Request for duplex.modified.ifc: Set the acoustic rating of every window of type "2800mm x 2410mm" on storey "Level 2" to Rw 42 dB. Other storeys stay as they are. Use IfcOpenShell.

First a look at what the model holds.

```python
import ifcopenshell
import ifcopenshell.util.element

model = ifcopenshell.open("duplex.modified.ifc")
print(model.schema)
storey = next(s for s in model.by_type("IfcBuildingStorey") if s.Name == "Level 2")
windows = [e for e in ifcopenshell.util.element.get_decomposition(storey) if e.is_a("IfcWindow")]
seen = {}
for e in windows:
    element_type = ifcopenshell.util.element.get_type(e)
    key = (element_type.Name if element_type != e and element_type else None, ifcopenshell.util.element.get_pset(e, "Pset_WindowCommon", "AcousticRating"))
    seen[key] = seen.get(key, 0) + 1
for (name, value), count in sorted(seen.items(), key=str):
    print(count, "x", name, "|", value)
```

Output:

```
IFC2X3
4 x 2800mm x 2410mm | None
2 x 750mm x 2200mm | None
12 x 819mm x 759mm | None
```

```python
import ifcopenshell
import ifcopenshell.api.pset
import ifcopenshell.util.element

model = ifcopenshell.open("duplex.modified.ifc")

storey = next(s for s in model.by_type("IfcBuildingStorey") if s.Name == "Level 2")
windows = [e for e in ifcopenshell.util.element.get_decomposition(storey) if e.is_a("IfcWindow")]

count = 0
for e in windows:
    element_type = ifcopenshell.util.element.get_type(e)
    if element_type in (None, e) or element_type.Name != "2800mm x 2410mm":
        continue
    # add_pset returns the element's existing set when there is one.
    pset = ifcopenshell.api.pset.add_pset(model, product=e, name="Pset_WindowCommon")
    ifcopenshell.api.pset.edit_pset(model, pset=pset, properties={"AcousticRating": "Rw 42 dB"})
    count += 1

print(count, "windows updated")

model.write("duplex.modified_edited.ifc")
```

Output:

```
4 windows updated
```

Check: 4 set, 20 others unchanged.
